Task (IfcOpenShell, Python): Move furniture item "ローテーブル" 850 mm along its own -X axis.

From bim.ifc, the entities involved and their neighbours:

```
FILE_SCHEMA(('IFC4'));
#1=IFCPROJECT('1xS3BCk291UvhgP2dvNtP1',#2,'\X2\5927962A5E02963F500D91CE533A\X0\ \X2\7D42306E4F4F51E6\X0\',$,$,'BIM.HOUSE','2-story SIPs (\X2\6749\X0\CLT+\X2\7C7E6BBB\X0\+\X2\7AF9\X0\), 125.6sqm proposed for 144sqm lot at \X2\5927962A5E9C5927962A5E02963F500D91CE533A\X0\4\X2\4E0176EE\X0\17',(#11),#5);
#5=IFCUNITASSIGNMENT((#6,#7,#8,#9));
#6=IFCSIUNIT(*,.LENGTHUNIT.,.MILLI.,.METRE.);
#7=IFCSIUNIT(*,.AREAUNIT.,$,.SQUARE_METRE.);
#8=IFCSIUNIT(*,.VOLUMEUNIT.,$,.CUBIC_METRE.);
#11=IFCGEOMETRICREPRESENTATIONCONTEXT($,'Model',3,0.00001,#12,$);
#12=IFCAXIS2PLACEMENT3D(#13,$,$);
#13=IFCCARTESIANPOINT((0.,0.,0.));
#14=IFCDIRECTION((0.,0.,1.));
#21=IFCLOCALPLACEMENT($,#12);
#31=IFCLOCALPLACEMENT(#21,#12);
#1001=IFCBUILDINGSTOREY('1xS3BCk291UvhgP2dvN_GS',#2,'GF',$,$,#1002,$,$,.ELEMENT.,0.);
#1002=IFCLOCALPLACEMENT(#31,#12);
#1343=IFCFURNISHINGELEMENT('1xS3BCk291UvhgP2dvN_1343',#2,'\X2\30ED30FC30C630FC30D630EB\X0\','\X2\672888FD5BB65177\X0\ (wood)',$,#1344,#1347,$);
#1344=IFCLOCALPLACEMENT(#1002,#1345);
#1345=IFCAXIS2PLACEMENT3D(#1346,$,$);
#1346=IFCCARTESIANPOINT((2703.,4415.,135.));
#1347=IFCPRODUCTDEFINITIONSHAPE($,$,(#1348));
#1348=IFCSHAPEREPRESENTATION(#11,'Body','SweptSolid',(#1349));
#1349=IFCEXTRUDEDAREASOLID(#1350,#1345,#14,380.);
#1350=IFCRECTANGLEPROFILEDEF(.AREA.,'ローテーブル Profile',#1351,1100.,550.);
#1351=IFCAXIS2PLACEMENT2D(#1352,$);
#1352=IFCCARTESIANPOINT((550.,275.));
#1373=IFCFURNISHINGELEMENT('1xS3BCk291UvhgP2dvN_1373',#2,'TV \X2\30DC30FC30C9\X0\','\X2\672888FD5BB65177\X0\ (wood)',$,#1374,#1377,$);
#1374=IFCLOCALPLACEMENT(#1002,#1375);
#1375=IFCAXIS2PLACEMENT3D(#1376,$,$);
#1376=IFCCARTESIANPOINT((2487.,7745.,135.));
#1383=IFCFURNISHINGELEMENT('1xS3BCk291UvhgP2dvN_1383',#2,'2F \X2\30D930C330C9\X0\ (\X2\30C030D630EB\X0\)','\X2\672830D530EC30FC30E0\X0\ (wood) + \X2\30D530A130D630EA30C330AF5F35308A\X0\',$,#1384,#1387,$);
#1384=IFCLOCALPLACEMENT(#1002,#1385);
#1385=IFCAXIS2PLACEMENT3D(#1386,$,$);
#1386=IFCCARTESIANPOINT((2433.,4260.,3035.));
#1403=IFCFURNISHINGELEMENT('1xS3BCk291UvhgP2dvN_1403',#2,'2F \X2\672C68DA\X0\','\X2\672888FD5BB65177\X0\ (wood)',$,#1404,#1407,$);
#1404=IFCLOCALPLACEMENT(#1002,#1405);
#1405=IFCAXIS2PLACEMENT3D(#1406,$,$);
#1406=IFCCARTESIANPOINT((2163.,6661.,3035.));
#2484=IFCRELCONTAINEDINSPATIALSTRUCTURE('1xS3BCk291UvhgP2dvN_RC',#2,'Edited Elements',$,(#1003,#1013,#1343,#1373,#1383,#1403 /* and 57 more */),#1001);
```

```python
import ifcopenshell
import ifcopenshell.api.geometry
import ifcopenshell.util.placement
import ifcopenshell.util.unit

model = ifcopenshell.open("bim.ifc")
unit_scale = ifcopenshell.util.unit.calculate_unit_scale(model)

item = model.by_guid("1xS3BCk291UvhgP2dvN_1343")
matrix = ifcopenshell.util.placement.get_local_placement(item.ObjectPlacement)
matrix[:3, 3] -= matrix[:3, 0] * 0.85 / unit_scale
ifcopenshell.api.geometry.edit_object_placement(model, product=item, matrix=matrix, is_si=False)

print(ifcopenshell.util.placement.get_local_placement(item.ObjectPlacement).round(3) + 0.0)

model.write("bim_rev.ifc")
```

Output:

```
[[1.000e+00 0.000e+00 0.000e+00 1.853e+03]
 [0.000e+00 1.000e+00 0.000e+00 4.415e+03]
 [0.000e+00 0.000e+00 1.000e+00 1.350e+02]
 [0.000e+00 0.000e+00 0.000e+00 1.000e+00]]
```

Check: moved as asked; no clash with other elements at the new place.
